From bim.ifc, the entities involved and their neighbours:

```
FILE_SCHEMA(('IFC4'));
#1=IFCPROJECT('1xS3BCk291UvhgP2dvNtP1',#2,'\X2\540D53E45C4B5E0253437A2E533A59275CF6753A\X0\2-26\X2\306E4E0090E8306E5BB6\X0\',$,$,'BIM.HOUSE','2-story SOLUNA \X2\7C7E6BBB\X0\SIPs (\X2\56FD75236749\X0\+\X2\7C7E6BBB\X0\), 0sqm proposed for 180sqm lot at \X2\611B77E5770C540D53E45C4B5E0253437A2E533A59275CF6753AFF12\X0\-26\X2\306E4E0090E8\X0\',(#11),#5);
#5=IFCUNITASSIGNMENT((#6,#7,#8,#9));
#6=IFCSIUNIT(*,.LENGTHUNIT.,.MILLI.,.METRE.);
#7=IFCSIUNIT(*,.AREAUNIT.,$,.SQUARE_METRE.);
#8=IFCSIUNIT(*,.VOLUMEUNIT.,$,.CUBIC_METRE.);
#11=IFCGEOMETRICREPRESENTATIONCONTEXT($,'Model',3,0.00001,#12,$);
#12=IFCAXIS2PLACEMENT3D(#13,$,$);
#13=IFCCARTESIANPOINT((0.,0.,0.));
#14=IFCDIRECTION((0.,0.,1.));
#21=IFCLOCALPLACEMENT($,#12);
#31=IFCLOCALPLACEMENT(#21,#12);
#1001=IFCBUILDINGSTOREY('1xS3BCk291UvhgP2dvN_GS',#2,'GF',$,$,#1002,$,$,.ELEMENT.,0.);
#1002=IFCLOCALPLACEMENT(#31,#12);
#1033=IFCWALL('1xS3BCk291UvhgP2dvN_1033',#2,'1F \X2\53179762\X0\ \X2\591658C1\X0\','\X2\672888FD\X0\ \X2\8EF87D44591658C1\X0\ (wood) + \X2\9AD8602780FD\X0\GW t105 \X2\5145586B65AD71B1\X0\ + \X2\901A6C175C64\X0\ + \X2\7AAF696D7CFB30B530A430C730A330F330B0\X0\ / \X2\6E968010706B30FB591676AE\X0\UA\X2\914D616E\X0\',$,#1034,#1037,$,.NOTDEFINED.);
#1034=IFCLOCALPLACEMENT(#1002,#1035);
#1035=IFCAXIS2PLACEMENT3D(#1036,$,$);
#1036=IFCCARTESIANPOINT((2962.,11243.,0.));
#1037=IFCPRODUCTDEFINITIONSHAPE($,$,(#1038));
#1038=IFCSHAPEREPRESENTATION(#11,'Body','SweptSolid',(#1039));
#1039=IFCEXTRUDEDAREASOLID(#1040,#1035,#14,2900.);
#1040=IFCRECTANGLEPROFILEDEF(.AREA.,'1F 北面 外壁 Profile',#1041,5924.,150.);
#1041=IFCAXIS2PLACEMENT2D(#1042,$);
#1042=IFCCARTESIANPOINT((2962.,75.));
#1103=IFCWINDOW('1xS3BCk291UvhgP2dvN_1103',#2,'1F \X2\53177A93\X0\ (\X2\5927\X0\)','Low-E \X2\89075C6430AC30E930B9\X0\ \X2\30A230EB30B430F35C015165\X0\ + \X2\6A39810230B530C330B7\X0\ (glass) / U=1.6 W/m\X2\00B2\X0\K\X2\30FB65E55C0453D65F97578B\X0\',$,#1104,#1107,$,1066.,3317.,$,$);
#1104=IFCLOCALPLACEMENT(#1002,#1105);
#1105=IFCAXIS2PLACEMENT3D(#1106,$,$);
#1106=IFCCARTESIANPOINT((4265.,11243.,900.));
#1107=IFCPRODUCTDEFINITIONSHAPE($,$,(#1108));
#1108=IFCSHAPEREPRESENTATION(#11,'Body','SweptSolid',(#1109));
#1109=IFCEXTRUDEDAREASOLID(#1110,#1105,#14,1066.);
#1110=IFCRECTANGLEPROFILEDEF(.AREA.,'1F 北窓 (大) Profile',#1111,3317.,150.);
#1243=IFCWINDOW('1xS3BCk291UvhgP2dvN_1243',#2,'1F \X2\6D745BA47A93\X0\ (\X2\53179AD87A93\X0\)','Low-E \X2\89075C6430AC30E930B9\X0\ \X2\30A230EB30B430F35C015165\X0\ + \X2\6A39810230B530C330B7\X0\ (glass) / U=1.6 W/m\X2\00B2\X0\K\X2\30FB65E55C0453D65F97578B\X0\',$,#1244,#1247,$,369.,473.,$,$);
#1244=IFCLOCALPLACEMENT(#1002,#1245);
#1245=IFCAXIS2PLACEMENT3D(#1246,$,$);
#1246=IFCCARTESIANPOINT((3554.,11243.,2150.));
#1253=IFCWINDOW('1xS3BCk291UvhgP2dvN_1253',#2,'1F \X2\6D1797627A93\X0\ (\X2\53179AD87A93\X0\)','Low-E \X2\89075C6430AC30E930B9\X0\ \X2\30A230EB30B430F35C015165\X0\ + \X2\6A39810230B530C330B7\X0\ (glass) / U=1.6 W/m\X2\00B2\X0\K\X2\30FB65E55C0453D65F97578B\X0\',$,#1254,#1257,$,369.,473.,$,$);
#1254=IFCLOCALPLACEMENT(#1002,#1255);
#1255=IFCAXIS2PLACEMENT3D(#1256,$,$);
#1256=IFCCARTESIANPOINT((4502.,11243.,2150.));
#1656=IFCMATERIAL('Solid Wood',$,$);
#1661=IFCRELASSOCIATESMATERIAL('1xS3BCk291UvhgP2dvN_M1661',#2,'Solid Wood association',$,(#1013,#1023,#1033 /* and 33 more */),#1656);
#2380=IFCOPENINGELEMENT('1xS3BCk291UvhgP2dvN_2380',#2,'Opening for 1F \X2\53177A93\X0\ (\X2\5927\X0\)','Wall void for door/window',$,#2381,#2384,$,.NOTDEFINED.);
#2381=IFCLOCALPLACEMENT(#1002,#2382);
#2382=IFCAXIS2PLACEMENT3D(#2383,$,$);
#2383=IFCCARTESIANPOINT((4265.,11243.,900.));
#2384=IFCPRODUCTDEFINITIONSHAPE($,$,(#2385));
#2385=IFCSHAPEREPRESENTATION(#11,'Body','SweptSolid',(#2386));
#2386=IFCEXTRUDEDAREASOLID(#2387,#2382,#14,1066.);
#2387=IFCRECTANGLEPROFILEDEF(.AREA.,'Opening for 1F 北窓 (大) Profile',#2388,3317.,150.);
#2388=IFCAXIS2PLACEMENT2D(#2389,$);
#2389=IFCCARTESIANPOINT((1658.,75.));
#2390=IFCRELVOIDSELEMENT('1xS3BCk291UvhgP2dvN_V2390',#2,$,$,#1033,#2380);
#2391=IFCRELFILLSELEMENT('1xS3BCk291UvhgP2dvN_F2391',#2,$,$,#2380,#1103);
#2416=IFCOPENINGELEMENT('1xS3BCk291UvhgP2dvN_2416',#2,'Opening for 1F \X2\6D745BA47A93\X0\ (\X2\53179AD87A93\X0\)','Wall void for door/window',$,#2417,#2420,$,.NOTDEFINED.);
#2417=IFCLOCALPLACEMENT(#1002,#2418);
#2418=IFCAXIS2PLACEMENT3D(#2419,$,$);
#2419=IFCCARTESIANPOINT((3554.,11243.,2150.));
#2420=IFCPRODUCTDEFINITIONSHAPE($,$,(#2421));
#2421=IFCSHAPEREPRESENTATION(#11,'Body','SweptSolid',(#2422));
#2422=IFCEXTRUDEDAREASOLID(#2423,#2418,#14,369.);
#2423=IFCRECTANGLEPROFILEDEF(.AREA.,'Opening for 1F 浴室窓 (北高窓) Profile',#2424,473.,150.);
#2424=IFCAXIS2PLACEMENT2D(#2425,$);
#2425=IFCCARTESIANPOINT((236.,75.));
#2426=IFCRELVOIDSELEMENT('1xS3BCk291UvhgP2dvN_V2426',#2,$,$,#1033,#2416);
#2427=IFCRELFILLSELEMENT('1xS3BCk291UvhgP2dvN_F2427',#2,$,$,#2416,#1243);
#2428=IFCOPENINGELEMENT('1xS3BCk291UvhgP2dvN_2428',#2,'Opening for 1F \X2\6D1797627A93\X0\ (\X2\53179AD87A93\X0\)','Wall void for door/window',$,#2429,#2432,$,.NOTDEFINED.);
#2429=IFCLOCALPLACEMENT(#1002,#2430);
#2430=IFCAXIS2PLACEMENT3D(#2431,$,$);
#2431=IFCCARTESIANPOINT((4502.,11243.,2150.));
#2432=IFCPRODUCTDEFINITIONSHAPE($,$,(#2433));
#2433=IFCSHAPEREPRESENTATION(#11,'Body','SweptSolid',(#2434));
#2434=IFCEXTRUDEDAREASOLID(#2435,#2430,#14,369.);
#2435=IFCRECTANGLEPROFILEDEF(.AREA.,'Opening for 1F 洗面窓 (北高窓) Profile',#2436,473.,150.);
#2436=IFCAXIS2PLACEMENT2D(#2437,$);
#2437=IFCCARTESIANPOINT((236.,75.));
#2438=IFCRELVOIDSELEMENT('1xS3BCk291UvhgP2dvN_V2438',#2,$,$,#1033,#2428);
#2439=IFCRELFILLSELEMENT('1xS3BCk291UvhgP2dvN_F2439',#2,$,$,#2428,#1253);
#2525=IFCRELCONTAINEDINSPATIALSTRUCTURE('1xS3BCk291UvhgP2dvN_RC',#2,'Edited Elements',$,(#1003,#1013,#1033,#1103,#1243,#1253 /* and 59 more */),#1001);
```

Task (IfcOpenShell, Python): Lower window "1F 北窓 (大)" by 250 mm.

```python
import numpy as np
import ifcopenshell
import ifcopenshell.api.geometry
import ifcopenshell.util.placement
import ifcopenshell.util.unit

model = ifcopenshell.open("bim.ifc")
unit_scale = ifcopenshell.util.unit.calculate_unit_scale(model)

window = model.by_id(1103)
opening = window.FillsVoids[0].RelatingOpeningElement
dz = -250.0

shift = np.array([0.0, 0.0, dz])
# The window is not placed relative to its opening, so move both.
for product in (opening, window):
    matrix = ifcopenshell.util.placement.get_local_placement(product.ObjectPlacement)
    matrix[:3, 3] += shift
    ifcopenshell.api.geometry.edit_object_placement(model, product=product, matrix=matrix, is_si=False)

print(f"moved by {dz * unit_scale:+.3f} m")

model.write("bim_v2.ifc")
```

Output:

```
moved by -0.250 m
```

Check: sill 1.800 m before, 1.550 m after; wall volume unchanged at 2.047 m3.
